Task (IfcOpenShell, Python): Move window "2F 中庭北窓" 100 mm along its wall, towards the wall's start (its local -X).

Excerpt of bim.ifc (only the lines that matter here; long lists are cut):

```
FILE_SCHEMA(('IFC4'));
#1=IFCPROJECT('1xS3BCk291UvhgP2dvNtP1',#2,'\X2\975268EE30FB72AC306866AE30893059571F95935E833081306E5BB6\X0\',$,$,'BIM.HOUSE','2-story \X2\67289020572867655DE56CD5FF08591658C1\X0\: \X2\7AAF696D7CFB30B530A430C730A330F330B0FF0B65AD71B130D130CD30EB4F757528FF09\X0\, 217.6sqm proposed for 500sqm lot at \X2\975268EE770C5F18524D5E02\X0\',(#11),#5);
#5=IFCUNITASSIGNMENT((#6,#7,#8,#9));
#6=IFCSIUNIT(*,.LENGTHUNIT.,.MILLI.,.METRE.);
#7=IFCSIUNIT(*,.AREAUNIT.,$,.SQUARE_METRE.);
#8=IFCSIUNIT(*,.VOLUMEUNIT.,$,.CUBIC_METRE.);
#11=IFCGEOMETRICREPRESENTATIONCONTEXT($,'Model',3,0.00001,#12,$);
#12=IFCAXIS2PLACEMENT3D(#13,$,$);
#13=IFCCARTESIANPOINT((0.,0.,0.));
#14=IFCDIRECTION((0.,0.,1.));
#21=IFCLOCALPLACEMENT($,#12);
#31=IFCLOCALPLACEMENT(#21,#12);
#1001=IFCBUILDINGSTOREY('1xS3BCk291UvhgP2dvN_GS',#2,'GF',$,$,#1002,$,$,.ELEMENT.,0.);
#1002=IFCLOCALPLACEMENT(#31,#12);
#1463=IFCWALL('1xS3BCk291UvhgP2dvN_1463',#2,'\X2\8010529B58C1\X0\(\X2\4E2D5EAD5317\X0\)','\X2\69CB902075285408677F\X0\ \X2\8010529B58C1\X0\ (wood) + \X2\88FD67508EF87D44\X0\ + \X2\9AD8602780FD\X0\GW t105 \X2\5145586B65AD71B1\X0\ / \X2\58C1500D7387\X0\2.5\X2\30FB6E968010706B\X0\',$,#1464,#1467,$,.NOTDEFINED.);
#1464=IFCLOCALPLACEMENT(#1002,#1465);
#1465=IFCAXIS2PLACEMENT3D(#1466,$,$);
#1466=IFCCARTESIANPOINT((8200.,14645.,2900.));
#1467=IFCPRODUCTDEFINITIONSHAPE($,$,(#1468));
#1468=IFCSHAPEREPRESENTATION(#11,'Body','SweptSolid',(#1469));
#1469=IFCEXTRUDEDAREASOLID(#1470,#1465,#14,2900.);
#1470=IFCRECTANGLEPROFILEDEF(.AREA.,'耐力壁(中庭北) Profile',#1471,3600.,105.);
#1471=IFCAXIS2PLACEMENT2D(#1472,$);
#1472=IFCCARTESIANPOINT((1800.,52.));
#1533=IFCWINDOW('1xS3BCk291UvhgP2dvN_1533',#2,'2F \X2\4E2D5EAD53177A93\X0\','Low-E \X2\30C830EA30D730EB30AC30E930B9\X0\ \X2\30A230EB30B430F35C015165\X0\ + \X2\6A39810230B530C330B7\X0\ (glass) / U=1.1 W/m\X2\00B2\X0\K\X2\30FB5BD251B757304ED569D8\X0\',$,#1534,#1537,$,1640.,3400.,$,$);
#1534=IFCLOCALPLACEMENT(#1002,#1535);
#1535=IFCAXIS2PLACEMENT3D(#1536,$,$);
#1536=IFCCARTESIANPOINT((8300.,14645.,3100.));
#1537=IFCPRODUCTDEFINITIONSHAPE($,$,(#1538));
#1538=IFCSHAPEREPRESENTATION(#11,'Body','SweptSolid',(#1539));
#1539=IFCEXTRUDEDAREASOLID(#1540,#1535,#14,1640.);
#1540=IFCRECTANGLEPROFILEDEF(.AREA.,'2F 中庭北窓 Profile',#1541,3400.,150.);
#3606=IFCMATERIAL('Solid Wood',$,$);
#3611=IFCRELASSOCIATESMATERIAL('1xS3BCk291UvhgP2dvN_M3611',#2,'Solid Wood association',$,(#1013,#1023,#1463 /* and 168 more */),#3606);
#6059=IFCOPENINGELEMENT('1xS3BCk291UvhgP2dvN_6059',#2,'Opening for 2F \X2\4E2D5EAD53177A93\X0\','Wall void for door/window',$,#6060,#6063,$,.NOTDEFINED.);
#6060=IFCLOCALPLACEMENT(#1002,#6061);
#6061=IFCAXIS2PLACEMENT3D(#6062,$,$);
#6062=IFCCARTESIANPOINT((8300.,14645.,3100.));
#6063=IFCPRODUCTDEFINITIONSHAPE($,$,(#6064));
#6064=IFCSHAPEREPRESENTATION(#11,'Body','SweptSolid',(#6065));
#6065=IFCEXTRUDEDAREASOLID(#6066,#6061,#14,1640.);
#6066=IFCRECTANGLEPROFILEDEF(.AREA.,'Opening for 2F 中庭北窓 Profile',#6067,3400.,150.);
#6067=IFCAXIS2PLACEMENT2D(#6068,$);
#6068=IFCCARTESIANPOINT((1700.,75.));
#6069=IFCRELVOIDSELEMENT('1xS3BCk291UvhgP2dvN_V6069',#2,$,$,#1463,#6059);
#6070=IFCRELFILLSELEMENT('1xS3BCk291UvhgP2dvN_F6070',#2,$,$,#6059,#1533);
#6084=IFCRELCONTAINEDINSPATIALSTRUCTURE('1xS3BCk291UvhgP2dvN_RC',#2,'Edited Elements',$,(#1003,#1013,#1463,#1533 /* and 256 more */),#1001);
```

```python
import ifcopenshell
import ifcopenshell.api.geometry
import ifcopenshell.util.placement
import ifcopenshell.util.unit

model = ifcopenshell.open("bim.ifc")
unit_scale = ifcopenshell.util.unit.calculate_unit_scale(model)

window = model.by_guid("1xS3BCk291UvhgP2dvN_1533")
opening = window.FillsVoids[0].RelatingOpeningElement
wall = opening.VoidsElements[0].RelatingBuildingElement

wall_matrix = ifcopenshell.util.placement.get_local_placement(wall.ObjectPlacement)
shift = wall_matrix[:3, 0] * -0.1 / unit_scale
before = ifcopenshell.util.placement.get_local_placement(window.ObjectPlacement)[:3, 3].copy()

# The window is not placed relative to its opening, so move both.
for product in (opening, window):
    matrix = ifcopenshell.util.placement.get_local_placement(product.ObjectPlacement)
    matrix[:3, 3] += shift
    ifcopenshell.api.geometry.edit_object_placement(model, product=product, matrix=matrix, is_si=False)

after = ifcopenshell.util.placement.get_local_placement(window.ObjectPlacement)[:3, 3]
print("window moved by", (after - before).round(3) + 0.0)

model.write("bim_v2.ifc")
```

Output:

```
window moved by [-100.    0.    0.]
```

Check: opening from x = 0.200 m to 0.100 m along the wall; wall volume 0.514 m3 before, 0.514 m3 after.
